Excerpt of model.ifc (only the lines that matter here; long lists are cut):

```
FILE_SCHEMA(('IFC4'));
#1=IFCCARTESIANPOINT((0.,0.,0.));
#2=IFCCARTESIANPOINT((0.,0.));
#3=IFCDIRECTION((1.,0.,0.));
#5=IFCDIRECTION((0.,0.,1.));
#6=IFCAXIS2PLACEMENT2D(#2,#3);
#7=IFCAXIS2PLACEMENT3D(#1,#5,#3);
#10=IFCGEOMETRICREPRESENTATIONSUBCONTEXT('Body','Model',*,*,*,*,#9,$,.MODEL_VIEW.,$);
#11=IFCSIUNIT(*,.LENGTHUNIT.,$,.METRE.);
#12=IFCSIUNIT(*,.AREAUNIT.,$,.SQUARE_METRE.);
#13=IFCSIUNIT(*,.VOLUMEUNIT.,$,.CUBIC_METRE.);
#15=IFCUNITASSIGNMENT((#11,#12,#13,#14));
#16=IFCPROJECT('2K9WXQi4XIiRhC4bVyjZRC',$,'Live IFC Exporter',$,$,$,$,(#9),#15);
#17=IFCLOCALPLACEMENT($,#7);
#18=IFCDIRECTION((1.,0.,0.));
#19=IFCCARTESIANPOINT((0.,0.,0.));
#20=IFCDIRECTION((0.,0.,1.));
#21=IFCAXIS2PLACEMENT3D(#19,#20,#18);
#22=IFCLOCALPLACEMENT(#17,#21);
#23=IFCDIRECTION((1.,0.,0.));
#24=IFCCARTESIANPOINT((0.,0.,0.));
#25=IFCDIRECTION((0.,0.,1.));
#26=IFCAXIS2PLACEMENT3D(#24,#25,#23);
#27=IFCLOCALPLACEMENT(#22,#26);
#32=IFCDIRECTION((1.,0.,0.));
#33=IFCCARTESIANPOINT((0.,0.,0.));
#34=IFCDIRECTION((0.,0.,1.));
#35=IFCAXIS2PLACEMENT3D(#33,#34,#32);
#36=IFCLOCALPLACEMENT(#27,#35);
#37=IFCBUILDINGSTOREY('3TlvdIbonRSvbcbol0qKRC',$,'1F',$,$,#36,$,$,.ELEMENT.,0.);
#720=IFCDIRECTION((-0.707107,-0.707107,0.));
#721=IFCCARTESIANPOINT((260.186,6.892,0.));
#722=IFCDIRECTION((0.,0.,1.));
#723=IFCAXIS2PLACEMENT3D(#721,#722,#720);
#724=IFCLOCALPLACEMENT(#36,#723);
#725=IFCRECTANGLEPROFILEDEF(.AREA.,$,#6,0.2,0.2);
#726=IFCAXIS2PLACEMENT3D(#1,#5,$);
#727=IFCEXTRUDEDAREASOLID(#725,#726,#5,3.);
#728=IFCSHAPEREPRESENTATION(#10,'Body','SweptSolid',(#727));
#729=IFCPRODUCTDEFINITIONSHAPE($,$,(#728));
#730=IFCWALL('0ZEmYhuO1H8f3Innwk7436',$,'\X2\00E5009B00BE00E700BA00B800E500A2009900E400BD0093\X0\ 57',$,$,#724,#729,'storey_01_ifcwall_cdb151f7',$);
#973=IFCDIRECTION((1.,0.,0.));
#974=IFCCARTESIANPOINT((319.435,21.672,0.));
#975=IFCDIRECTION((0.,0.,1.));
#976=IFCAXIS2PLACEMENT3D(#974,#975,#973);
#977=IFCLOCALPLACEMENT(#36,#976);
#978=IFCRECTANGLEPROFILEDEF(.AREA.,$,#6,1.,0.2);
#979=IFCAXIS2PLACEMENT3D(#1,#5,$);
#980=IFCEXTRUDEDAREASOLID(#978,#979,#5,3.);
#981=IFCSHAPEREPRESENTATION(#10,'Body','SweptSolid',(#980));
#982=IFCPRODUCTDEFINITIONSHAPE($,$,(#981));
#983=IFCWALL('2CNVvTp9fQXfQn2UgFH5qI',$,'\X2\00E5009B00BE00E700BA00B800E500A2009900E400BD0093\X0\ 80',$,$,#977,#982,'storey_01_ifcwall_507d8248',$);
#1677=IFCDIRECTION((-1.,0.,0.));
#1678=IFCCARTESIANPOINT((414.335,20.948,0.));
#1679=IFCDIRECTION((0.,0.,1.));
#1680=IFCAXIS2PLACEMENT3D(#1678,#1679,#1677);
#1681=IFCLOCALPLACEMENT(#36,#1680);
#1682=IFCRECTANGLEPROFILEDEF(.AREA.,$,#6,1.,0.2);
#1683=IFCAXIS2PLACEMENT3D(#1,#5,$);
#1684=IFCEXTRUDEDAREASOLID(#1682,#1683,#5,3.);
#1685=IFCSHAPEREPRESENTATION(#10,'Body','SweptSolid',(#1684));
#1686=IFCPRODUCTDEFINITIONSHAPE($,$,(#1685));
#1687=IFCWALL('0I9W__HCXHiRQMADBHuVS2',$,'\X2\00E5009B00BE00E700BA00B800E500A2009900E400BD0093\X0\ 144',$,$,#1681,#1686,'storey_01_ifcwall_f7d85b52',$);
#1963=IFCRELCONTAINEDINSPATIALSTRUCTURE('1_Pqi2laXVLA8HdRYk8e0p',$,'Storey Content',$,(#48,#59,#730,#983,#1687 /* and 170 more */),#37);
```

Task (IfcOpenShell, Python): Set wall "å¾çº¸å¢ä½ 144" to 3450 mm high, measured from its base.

```python
import ifcopenshell
import ifcopenshell.geom
import ifcopenshell.util.representation
import ifcopenshell.util.shape

model = ifcopenshell.open("model.ifc")
settings = ifcopenshell.geom.settings()


def volume(element):
    """Net volume in cubic metres, openings subtracted."""
    shape = ifcopenshell.geom.create_shape(settings, element)
    return ifcopenshell.util.shape.get_volume(shape.geometry)


wall = model.by_guid("0I9W__HCXHiRQMADBHuVS2")
before = volume(wall)

body = ifcopenshell.util.representation.get_representation(wall, "Model", "Body")
solid = body.Items[0]
old_height = solid.Depth
solid.Depth = 3.45
after = volume(wall)

print(f"height {old_height:g} -> {solid.Depth:g}, volume {before:.3f} -> {after:.3f} m3")

model.write("model_updated.ifc")
```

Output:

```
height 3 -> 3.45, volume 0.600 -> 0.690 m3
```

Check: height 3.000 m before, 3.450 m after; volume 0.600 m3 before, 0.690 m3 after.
